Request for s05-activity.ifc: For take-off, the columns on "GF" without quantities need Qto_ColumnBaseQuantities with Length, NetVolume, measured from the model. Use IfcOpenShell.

First a look at what the model holds.

```python
import ifcopenshell
import ifcopenshell.util.element
import ifcopenshell.util.unit

model = ifcopenshell.open("s05-activity.ifc")
print(model.schema)
for unit_type in ("LENGTHUNIT", "AREAUNIT", "VOLUMEUNIT"):
    print(unit_type, ifcopenshell.util.unit.calculate_unit_scale(model, unit_type))
storey = next(s for s in model.by_type("IfcBuildingStorey") if s.Name == "GF")
columns = [e for e in ifcopenshell.util.element.get_decomposition(storey) if e.is_a("IfcColumn")]
for e in sorted(columns, key=lambda e: e.id()):
    print(e.id(), e.is_a(), e.Name, list(ifcopenshell.util.element.get_psets(e, qtos_only=True)), sep=" | ")
```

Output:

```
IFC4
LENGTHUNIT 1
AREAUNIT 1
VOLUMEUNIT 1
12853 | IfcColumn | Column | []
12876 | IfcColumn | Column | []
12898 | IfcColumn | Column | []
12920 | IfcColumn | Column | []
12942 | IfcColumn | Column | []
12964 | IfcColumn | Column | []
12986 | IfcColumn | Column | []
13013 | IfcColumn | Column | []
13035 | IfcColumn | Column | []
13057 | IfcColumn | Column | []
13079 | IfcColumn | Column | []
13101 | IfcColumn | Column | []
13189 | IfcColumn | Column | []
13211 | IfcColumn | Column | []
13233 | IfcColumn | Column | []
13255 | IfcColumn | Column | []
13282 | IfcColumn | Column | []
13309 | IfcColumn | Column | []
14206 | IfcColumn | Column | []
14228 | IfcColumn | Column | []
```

```python
import ifcopenshell
import ifcopenshell.api.pset
import ifcopenshell.geom
import ifcopenshell.util.element
import ifcopenshell.util.shape
import ifcopenshell.util.unit

model = ifcopenshell.open("s05-activity.ifc")
unit_scale = ifcopenshell.util.unit.calculate_unit_scale(model)
volume_scale = ifcopenshell.util.unit.calculate_unit_scale(model, "VOLUMEUNIT")
settings = ifcopenshell.geom.settings()

storey = next(s for s in model.by_type("IfcBuildingStorey") if s.Name == "GF")
columns = [e for e in ifcopenshell.util.element.get_decomposition(storey) if e.is_a("IfcColumn")]

for e in sorted(columns, key=lambda e: e.id()):
    if ifcopenshell.util.element.get_psets(e, qtos_only=True, should_inherit=False):
        continue
    # Geometry comes back in metres, in the element's own axes.
    shape = ifcopenshell.geom.create_shape(settings, e)
    values = {
        "Length": ifcopenshell.util.shape.get_z(shape.geometry) / unit_scale,
        "NetVolume": ifcopenshell.util.shape.get_volume(shape.geometry) / volume_scale,
    }
    qto = ifcopenshell.api.pset.add_qto(model, product=e, name="Qto_ColumnBaseQuantities")
    ifcopenshell.api.pset.edit_qto(model, qto=qto, properties=values)
    print(e.id(), {k: round(v, 3) for k, v in values.items()})

model.write("s05-activity_rev.ifc")
```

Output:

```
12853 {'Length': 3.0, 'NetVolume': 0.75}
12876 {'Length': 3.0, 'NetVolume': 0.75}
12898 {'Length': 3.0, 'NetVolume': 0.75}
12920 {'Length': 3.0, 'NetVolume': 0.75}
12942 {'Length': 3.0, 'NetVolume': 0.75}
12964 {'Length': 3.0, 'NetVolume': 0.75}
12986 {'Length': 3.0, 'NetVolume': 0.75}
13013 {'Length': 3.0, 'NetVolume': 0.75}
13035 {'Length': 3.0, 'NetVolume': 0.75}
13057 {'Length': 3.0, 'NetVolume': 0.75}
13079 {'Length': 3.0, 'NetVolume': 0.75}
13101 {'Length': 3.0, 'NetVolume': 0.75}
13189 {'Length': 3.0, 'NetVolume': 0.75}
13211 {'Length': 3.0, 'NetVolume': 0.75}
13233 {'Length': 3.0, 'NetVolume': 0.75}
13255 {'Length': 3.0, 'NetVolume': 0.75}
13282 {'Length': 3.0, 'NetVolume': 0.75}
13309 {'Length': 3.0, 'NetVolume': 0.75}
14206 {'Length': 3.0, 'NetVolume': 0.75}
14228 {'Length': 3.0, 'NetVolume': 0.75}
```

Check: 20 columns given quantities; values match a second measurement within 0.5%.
